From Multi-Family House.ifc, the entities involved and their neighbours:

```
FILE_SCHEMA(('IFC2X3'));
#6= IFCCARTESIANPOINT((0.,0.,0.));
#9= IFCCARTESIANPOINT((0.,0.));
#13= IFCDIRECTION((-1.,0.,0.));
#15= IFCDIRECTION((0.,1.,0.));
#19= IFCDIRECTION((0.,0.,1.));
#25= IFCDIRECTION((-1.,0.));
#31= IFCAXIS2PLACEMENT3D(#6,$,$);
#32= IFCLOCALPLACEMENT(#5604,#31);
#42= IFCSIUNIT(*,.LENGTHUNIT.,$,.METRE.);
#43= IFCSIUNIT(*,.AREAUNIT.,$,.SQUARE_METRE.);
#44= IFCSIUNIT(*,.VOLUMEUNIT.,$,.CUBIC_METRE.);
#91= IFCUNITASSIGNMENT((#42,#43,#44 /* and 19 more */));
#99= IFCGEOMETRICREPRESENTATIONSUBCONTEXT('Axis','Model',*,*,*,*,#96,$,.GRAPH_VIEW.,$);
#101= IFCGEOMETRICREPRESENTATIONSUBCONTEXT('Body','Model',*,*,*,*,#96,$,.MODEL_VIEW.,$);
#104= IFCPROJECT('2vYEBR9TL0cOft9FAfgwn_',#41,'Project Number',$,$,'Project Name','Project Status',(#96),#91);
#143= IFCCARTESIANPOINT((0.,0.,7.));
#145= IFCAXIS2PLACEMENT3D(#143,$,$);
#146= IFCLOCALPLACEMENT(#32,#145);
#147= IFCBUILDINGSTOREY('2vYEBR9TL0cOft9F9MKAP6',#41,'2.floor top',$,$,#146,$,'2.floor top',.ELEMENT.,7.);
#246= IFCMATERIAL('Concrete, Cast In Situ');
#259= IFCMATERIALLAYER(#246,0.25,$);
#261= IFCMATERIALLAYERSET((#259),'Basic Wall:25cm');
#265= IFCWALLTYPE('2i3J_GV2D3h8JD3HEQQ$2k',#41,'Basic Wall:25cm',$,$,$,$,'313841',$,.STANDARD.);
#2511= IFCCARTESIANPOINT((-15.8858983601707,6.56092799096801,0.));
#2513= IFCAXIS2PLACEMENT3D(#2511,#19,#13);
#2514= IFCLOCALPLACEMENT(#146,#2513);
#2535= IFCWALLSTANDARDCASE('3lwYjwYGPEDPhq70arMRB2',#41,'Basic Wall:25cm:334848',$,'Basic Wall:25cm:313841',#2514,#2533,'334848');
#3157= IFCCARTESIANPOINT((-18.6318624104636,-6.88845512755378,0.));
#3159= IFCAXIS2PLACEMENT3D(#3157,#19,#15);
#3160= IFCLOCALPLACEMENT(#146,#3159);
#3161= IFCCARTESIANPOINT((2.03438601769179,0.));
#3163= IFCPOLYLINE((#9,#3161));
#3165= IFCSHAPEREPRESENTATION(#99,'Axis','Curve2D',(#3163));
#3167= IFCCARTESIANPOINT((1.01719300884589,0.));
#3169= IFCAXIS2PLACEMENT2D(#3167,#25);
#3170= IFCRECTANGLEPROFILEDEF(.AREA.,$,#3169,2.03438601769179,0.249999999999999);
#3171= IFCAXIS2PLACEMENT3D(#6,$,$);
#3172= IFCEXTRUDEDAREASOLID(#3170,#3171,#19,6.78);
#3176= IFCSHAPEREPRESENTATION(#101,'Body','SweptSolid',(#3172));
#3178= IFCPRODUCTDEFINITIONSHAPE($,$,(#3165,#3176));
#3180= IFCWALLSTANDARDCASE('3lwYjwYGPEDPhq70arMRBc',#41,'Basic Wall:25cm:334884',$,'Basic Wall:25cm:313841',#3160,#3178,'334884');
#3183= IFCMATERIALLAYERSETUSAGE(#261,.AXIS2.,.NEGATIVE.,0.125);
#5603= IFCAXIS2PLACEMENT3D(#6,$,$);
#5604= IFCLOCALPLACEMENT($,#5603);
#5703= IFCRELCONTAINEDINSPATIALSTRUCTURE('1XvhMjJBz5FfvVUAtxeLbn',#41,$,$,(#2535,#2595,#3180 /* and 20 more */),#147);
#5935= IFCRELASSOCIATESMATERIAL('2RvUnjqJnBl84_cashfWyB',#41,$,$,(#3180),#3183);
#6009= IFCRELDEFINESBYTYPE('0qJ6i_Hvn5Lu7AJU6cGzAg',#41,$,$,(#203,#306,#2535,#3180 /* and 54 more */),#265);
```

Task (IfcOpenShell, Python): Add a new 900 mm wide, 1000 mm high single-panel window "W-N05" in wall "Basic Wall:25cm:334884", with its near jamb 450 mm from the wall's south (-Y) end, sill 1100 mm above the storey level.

```python
import numpy as np
import ifcopenshell
import ifcopenshell.api.feature
import ifcopenshell.api.geometry
import ifcopenshell.api.root
import ifcopenshell.api.spatial
import ifcopenshell.api.type
import ifcopenshell.geom
import ifcopenshell.util.element
import ifcopenshell.util.placement
import ifcopenshell.util.representation
import ifcopenshell.util.shape
import ifcopenshell.util.unit

model = ifcopenshell.open("Multi-Family House.ifc")
unit_scale = ifcopenshell.util.unit.calculate_unit_scale(model)
settings = ifcopenshell.geom.settings()


def volume(element):
    """Net volume in cubic metres, openings subtracted."""
    shape = ifcopenshell.geom.create_shape(settings, element)
    return ifcopenshell.util.shape.get_volume(shape.geometry)


wall = model.by_guid("3lwYjwYGPEDPhq70arMRBc")
storey = ifcopenshell.util.element.get_container(wall, ifc_class="IfcBuildingStorey")
context = ifcopenshell.util.representation.get_context(model, "Model", "Body", "MODEL_VIEW")
before = volume(wall)

width, height, from_end, sill = 0.9, 1, 0.45, 1.1  # metres

# The wall runs along its own X axis, and the end named is its -X end.
wall_shape = ifcopenshell.geom.create_shape(settings, wall)
x, y, z = ifcopenshell.util.shape.get_vertices(wall_shape.geometry).T
start = x.min() + from_end
face, thickness = float(y.min()), float(y.max() - y.min())
wall_matrix = ifcopenshell.util.placement.get_local_placement(wall.ObjectPlacement)
level = ifcopenshell.util.placement.get_local_placement(storey.ObjectPlacement)[2, 3]


def in_wall(x, y):
    """Placement at x, y metres in the wall's axes, at sill height."""
    matrix = wall_matrix.copy()
    matrix[:, 3] = wall_matrix @ np.array([x / unit_scale, y / unit_scale, 0.0, 1.0])
    matrix[2, 3] = level + sill / unit_scale
    return matrix


# Opening: a box that overshoots both wall faces by 50 mm.
opening = ifcopenshell.api.root.create_entity(model, ifc_class="IfcOpeningElement")
box = ifcopenshell.api.geometry.add_wall_representation(
    model, context=context, length=width, height=height, thickness=thickness + 0.1
)
ifcopenshell.api.geometry.assign_representation(model, product=opening, representation=box)
ifcopenshell.api.geometry.edit_object_placement(model, product=opening, matrix=in_wall(start, face - 0.05), is_si=False)
ifcopenshell.api.feature.add_feature(model, feature=opening, element=wall)

window = ifcopenshell.api.root.create_entity(model, ifc_class="IfcWindow", name="W-N05")
window.OverallWidth, window.OverallHeight = width / unit_scale, height / unit_scale
body = ifcopenshell.api.geometry.add_window_representation(
    model,
    context=context,
    overall_width=window.OverallWidth,
    overall_height=window.OverallHeight,
    partition_type="SINGLE_PANEL",
)
ifcopenshell.api.geometry.assign_representation(model, product=window, representation=body)
ifcopenshell.api.spatial.assign_container(model, products=[window], relating_structure=storey)
fills = ifcopenshell.api.feature.add_filling(model, opening=opening, element=window)
fills.OwnerHistory = window.OwnerHistory  # required in IFC2X3

# IFC2X3 keeps the operation on the window style.
style = ifcopenshell.api.root.create_entity(model, ifc_class="IfcWindowStyle", name="W-N05")
style.OperationType, style.ConstructionType = "SINGLE_PANEL", "NOTDEFINED"
style.ParameterTakesPrecedence = style.Sizeable = False
ifcopenshell.api.type.assign_type(model, related_objects=[window], relating_type=style)

# Centre the window in the wall's thickness.
ifcopenshell.api.geometry.edit_object_placement(model, product=window, matrix=in_wall(start, face), is_si=False)
window_shape = ifcopenshell.geom.create_shape(settings, window)
depth = ifcopenshell.util.shape.get_vertices(window_shape.geometry)[:, 1]
offset = face + thickness / 2 - (depth.min() + depth.max()) / 2
ifcopenshell.api.geometry.edit_object_placement(model, product=window, matrix=in_wall(start, offset), is_si=False)

after = volume(wall)

print(f"wall volume {before:.3f} -> {after:.3f} m3")

model.write("Multi-Family House_v2.ifc")
```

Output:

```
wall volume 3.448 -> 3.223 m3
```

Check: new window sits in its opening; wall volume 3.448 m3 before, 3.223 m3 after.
